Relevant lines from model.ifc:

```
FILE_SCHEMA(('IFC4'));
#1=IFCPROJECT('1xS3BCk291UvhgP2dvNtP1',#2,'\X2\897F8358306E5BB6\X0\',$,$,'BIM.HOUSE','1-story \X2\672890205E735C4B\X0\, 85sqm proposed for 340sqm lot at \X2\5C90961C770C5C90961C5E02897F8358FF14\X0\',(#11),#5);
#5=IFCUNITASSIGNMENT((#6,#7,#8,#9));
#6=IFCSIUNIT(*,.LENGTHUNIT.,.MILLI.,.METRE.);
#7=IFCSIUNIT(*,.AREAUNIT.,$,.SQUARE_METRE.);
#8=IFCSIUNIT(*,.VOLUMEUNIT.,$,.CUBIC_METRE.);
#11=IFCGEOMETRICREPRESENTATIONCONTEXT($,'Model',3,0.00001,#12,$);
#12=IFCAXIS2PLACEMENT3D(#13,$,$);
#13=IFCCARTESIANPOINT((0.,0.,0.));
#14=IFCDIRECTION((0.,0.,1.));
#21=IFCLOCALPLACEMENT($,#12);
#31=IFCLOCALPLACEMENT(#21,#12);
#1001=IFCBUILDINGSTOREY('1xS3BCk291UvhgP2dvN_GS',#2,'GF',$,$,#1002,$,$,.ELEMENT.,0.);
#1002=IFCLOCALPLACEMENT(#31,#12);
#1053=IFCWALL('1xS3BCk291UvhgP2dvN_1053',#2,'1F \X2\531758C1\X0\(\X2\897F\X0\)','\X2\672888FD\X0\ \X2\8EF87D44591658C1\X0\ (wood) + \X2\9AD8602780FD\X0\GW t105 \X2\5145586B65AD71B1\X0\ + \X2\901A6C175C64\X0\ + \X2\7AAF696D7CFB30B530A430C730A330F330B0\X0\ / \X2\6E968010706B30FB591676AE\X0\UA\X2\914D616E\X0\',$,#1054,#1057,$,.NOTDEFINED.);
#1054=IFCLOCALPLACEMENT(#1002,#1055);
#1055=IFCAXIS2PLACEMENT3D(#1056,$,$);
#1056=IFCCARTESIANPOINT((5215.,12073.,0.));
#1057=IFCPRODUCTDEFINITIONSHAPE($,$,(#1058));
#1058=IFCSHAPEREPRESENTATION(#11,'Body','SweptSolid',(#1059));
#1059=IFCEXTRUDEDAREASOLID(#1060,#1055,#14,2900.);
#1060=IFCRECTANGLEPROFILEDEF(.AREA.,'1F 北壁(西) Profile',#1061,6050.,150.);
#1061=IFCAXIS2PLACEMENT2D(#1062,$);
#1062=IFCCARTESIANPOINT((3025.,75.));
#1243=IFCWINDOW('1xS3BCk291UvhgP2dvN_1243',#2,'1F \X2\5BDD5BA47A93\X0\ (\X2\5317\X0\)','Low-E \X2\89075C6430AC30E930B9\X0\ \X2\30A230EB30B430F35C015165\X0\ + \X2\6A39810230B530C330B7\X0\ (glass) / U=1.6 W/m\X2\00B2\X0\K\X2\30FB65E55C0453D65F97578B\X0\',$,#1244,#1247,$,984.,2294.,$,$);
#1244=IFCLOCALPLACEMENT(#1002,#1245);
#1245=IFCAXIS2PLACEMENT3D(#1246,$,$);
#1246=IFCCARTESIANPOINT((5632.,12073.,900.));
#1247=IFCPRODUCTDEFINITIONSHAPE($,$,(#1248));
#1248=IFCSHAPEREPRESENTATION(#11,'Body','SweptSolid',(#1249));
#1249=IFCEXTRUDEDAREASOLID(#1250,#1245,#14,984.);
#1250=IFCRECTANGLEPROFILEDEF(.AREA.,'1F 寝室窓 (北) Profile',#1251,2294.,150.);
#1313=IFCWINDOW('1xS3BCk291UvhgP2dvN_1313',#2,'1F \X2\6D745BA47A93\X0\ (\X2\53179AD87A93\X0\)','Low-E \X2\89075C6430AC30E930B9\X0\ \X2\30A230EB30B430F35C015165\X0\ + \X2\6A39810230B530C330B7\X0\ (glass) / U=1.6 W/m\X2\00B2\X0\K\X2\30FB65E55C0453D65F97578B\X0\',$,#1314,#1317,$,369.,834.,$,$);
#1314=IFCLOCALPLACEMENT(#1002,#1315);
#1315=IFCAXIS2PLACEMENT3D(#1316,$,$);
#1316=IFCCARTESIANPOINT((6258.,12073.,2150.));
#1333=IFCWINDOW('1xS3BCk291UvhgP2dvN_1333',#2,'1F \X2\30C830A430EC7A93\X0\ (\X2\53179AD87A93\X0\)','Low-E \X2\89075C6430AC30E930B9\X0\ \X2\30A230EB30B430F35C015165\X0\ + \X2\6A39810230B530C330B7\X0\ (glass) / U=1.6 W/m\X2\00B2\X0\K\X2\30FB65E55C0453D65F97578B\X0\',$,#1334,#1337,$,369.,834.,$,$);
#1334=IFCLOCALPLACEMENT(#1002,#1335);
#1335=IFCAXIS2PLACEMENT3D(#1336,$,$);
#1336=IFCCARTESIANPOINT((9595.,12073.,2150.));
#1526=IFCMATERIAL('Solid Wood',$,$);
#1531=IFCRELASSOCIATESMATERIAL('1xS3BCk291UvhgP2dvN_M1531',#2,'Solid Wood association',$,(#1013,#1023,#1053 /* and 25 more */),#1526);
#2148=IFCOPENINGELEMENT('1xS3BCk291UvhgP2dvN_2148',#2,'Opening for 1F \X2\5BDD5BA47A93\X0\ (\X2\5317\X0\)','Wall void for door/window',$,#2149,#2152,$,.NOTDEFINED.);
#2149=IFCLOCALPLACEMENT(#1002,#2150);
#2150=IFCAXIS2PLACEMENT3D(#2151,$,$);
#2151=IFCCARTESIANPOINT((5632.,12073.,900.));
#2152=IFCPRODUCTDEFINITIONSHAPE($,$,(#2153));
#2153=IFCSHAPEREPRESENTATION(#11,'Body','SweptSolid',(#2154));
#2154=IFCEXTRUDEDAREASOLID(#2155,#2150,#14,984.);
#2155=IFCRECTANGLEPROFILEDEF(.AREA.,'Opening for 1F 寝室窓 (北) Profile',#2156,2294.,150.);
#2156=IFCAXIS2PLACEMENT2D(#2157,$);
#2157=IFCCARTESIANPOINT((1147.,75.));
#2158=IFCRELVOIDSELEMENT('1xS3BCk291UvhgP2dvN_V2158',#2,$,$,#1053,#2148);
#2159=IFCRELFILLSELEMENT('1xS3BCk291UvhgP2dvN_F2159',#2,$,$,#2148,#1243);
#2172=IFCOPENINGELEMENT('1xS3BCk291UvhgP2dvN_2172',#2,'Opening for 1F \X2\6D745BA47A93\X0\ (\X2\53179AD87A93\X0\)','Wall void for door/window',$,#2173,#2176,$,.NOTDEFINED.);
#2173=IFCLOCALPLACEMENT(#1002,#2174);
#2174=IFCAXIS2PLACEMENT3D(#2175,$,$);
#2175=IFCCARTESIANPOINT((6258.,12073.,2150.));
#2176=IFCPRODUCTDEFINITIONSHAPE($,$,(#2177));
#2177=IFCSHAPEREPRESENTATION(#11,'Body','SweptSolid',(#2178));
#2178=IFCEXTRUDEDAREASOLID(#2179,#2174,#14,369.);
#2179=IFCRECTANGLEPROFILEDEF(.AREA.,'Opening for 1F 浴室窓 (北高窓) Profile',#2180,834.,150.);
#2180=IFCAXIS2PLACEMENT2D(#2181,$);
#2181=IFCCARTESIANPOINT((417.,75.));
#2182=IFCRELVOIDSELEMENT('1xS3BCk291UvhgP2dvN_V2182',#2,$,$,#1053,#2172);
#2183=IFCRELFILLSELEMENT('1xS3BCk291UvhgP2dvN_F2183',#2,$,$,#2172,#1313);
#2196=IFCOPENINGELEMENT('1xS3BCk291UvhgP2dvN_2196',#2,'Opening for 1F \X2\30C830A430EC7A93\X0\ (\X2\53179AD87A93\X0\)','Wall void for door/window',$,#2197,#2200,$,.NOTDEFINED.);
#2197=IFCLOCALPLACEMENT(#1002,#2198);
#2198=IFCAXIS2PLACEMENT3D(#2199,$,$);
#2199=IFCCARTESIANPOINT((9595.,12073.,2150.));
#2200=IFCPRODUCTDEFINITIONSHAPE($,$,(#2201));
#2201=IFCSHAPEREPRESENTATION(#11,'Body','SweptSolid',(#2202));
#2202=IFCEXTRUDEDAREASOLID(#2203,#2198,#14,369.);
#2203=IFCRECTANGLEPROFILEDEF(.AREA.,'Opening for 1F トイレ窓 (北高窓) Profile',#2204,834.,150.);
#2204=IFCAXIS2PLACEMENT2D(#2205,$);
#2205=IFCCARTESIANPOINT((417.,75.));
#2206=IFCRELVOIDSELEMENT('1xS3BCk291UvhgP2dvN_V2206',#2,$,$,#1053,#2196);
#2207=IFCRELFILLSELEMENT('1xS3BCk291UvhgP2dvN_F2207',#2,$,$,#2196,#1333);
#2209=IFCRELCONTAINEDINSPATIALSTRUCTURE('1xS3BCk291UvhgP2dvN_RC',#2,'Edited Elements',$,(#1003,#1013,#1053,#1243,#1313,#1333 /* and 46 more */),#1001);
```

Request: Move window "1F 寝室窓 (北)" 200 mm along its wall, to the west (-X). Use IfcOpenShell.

```python
import ifcopenshell
import ifcopenshell.api.geometry
import ifcopenshell.util.placement
import ifcopenshell.util.unit

model = ifcopenshell.open("model.ifc")
unit_scale = ifcopenshell.util.unit.calculate_unit_scale(model)

window = model.by_guid("1xS3BCk291UvhgP2dvN_1243")
opening = window.FillsVoids[0].RelatingOpeningElement
wall = opening.VoidsElements[0].RelatingBuildingElement

wall_matrix = ifcopenshell.util.placement.get_local_placement(wall.ObjectPlacement)
shift = wall_matrix[:3, 0] * -0.2 / unit_scale
before = ifcopenshell.util.placement.get_local_placement(window.ObjectPlacement)[:3, 3].copy()

# The window is not placed relative to its opening, so move both.
for product in (opening, window):
    matrix = ifcopenshell.util.placement.get_local_placement(product.ObjectPlacement)
    matrix[:3, 3] += shift
    ifcopenshell.api.geometry.edit_object_placement(model, product=product, matrix=matrix, is_si=False)

after = ifcopenshell.util.placement.get_local_placement(window.ObjectPlacement)[:3, 3]
print("window moved by", (after - before).round(3) + 0.0)

model.write("model_edited.ifc")
```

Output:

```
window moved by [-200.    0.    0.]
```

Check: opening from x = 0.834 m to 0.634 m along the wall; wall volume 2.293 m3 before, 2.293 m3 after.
